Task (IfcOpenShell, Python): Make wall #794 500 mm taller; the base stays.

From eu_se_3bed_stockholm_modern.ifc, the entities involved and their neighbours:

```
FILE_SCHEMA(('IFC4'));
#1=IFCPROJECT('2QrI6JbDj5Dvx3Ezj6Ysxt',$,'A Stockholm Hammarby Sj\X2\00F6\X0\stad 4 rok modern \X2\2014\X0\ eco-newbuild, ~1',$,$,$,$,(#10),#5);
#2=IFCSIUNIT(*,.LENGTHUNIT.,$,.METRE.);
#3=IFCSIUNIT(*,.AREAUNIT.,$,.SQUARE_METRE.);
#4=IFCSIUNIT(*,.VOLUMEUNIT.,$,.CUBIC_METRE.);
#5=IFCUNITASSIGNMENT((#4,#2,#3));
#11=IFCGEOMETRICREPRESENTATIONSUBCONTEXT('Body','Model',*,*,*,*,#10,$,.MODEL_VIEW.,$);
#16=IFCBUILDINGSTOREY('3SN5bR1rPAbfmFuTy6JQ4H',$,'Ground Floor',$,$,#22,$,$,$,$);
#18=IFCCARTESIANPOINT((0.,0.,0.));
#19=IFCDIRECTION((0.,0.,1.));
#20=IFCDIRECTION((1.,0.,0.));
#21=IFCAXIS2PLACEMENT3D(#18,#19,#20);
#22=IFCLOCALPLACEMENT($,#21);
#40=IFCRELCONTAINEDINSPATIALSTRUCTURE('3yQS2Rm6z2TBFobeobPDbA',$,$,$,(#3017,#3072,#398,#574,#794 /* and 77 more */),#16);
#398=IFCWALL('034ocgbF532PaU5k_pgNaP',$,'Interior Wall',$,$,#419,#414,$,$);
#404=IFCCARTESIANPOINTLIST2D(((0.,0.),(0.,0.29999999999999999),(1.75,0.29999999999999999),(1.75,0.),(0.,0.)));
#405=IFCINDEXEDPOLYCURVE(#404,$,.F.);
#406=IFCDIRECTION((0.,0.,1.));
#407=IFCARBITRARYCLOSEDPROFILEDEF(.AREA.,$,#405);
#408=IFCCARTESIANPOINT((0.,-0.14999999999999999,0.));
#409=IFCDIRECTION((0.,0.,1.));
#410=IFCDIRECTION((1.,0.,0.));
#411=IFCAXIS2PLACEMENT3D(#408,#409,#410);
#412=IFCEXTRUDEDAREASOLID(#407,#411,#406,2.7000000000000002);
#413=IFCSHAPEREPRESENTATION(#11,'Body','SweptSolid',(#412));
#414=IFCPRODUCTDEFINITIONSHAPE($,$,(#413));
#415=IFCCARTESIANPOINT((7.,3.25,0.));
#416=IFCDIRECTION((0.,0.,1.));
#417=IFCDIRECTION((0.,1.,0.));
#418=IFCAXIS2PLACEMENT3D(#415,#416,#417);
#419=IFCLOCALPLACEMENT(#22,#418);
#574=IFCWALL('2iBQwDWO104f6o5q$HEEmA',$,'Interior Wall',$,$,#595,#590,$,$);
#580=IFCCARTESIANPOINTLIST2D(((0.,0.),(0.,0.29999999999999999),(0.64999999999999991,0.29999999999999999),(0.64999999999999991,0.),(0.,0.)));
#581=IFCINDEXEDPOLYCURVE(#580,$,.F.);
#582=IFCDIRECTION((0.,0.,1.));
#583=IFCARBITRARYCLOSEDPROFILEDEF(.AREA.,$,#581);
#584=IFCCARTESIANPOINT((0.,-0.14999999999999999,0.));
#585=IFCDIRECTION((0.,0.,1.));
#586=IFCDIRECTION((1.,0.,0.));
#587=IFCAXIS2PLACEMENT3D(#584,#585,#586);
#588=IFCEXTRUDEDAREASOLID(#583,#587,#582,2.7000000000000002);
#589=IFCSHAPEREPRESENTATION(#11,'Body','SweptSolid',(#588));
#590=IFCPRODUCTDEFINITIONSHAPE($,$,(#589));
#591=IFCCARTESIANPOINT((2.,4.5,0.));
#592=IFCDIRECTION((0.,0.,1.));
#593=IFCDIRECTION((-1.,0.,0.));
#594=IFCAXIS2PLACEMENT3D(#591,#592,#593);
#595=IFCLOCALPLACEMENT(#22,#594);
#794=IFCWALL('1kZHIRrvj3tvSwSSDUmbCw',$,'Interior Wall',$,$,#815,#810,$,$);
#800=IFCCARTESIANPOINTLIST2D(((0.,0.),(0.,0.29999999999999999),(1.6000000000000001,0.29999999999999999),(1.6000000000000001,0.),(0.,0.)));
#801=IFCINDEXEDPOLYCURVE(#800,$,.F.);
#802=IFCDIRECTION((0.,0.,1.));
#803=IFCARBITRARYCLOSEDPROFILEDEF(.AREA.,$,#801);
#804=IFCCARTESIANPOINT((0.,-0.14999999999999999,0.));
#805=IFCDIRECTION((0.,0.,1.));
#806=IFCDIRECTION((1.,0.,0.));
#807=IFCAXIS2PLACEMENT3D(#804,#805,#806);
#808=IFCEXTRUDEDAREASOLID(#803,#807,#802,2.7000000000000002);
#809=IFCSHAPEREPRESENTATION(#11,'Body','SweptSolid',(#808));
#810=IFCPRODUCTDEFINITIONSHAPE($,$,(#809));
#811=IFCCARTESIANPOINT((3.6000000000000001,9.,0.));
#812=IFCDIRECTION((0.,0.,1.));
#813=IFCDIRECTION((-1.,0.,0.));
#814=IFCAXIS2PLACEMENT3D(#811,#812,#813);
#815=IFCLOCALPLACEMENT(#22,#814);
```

```python
import ifcopenshell
import ifcopenshell.geom
import ifcopenshell.util.representation
import ifcopenshell.util.shape

model = ifcopenshell.open("eu_se_3bed_stockholm_modern.ifc")
settings = ifcopenshell.geom.settings()


def volume(element):
    """Net volume in cubic metres, openings subtracted."""
    shape = ifcopenshell.geom.create_shape(settings, element)
    return ifcopenshell.util.shape.get_volume(shape.geometry)


wall = model.by_guid("1kZHIRrvj3tvSwSSDUmbCw")
before = volume(wall)

body = ifcopenshell.util.representation.get_representation(wall, "Model", "Body")
solid = body.Items[0]
old_height = solid.Depth
solid.Depth += 0.5
after = volume(wall)

print(f"height {old_height:g} -> {solid.Depth:g}, volume {before:.3f} -> {after:.3f} m3")

model.write("eu_se_3bed_stockholm_modern_edited.ifc")
```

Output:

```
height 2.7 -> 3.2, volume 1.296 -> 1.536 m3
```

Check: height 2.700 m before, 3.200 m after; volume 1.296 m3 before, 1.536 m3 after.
